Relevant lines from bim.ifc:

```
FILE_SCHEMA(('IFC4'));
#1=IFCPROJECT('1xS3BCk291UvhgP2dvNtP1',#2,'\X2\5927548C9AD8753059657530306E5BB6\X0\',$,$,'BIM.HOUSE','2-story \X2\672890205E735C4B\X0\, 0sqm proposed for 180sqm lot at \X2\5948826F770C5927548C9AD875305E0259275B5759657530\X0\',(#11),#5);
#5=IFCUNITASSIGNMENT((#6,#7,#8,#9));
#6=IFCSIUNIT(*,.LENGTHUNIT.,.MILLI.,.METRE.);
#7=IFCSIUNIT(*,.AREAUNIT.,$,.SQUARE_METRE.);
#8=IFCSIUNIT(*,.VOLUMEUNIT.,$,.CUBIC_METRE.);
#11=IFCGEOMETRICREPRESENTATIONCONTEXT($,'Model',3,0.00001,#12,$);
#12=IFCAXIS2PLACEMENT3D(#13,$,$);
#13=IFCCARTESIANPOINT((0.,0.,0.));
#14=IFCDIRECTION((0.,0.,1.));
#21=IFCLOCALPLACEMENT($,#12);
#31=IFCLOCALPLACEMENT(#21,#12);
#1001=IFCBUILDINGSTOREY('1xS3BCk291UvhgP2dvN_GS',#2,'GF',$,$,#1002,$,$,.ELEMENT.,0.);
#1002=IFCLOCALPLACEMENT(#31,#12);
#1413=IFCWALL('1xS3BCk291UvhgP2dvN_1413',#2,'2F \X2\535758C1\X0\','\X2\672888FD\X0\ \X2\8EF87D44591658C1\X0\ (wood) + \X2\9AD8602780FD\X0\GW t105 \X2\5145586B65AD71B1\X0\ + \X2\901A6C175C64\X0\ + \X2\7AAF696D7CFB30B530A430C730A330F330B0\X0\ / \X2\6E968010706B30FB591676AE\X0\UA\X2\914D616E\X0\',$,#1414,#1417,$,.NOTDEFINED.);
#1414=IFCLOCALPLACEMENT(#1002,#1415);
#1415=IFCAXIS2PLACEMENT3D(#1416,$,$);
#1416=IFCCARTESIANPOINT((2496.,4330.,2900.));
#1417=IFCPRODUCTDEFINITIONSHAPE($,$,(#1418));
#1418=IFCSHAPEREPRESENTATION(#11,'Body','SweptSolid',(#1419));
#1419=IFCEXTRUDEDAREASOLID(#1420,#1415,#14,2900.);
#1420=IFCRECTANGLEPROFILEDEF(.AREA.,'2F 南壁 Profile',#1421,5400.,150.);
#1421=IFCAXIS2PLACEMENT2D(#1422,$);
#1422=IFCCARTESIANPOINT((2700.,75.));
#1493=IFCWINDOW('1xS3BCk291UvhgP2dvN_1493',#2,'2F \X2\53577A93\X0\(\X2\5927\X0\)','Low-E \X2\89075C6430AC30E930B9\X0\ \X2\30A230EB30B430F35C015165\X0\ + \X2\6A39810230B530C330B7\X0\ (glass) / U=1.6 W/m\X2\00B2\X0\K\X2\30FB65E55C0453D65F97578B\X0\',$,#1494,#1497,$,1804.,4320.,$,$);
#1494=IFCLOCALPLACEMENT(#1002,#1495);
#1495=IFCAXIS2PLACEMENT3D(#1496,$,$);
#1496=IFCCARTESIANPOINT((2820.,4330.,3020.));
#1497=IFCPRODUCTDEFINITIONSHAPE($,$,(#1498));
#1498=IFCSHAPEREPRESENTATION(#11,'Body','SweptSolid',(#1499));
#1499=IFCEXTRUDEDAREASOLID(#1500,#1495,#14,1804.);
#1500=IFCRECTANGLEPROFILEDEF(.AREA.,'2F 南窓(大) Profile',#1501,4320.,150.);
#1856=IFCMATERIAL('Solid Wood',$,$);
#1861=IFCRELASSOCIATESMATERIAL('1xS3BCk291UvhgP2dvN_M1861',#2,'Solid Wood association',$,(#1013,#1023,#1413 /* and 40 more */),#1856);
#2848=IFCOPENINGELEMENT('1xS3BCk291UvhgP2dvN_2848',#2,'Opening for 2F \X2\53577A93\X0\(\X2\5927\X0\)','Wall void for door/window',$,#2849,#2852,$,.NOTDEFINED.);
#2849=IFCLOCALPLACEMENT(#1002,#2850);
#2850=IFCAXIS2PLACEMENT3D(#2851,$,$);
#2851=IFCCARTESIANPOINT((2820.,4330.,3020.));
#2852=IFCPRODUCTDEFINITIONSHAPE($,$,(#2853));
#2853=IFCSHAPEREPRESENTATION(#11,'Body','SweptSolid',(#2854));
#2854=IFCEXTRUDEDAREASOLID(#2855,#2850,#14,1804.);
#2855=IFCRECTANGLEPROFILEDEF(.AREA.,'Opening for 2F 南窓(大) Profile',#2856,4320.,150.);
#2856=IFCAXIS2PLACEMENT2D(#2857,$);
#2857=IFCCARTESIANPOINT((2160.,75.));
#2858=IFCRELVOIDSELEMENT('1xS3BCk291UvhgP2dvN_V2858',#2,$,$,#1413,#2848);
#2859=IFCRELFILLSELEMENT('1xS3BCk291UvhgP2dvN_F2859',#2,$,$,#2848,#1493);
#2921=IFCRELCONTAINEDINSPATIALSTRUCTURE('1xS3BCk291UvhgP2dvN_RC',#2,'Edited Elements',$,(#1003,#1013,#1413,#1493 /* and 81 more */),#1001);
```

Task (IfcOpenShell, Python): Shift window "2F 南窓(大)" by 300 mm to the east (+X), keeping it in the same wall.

```python
import ifcopenshell
import ifcopenshell.api.geometry
import ifcopenshell.util.placement
import ifcopenshell.util.unit

model = ifcopenshell.open("bim.ifc")
unit_scale = ifcopenshell.util.unit.calculate_unit_scale(model)

window = model.by_guid("1xS3BCk291UvhgP2dvN_1493")
opening = window.FillsVoids[0].RelatingOpeningElement
wall = opening.VoidsElements[0].RelatingBuildingElement

wall_matrix = ifcopenshell.util.placement.get_local_placement(wall.ObjectPlacement)
shift = wall_matrix[:3, 0] * 0.3 / unit_scale
before = ifcopenshell.util.placement.get_local_placement(window.ObjectPlacement)[:3, 3].copy()

# The window is not placed relative to its opening, so move both.
for product in (opening, window):
    matrix = ifcopenshell.util.placement.get_local_placement(product.ObjectPlacement)
    matrix[:3, 3] += shift
    ifcopenshell.api.geometry.edit_object_placement(model, product=product, matrix=matrix, is_si=False)

after = ifcopenshell.util.placement.get_local_placement(window.ObjectPlacement)[:3, 3]
print("window moved by", (after - before).round(3) + 0.0)

model.write("bim_v2.ifc")
```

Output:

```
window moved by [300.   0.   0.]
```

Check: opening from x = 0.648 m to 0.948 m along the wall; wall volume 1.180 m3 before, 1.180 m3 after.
